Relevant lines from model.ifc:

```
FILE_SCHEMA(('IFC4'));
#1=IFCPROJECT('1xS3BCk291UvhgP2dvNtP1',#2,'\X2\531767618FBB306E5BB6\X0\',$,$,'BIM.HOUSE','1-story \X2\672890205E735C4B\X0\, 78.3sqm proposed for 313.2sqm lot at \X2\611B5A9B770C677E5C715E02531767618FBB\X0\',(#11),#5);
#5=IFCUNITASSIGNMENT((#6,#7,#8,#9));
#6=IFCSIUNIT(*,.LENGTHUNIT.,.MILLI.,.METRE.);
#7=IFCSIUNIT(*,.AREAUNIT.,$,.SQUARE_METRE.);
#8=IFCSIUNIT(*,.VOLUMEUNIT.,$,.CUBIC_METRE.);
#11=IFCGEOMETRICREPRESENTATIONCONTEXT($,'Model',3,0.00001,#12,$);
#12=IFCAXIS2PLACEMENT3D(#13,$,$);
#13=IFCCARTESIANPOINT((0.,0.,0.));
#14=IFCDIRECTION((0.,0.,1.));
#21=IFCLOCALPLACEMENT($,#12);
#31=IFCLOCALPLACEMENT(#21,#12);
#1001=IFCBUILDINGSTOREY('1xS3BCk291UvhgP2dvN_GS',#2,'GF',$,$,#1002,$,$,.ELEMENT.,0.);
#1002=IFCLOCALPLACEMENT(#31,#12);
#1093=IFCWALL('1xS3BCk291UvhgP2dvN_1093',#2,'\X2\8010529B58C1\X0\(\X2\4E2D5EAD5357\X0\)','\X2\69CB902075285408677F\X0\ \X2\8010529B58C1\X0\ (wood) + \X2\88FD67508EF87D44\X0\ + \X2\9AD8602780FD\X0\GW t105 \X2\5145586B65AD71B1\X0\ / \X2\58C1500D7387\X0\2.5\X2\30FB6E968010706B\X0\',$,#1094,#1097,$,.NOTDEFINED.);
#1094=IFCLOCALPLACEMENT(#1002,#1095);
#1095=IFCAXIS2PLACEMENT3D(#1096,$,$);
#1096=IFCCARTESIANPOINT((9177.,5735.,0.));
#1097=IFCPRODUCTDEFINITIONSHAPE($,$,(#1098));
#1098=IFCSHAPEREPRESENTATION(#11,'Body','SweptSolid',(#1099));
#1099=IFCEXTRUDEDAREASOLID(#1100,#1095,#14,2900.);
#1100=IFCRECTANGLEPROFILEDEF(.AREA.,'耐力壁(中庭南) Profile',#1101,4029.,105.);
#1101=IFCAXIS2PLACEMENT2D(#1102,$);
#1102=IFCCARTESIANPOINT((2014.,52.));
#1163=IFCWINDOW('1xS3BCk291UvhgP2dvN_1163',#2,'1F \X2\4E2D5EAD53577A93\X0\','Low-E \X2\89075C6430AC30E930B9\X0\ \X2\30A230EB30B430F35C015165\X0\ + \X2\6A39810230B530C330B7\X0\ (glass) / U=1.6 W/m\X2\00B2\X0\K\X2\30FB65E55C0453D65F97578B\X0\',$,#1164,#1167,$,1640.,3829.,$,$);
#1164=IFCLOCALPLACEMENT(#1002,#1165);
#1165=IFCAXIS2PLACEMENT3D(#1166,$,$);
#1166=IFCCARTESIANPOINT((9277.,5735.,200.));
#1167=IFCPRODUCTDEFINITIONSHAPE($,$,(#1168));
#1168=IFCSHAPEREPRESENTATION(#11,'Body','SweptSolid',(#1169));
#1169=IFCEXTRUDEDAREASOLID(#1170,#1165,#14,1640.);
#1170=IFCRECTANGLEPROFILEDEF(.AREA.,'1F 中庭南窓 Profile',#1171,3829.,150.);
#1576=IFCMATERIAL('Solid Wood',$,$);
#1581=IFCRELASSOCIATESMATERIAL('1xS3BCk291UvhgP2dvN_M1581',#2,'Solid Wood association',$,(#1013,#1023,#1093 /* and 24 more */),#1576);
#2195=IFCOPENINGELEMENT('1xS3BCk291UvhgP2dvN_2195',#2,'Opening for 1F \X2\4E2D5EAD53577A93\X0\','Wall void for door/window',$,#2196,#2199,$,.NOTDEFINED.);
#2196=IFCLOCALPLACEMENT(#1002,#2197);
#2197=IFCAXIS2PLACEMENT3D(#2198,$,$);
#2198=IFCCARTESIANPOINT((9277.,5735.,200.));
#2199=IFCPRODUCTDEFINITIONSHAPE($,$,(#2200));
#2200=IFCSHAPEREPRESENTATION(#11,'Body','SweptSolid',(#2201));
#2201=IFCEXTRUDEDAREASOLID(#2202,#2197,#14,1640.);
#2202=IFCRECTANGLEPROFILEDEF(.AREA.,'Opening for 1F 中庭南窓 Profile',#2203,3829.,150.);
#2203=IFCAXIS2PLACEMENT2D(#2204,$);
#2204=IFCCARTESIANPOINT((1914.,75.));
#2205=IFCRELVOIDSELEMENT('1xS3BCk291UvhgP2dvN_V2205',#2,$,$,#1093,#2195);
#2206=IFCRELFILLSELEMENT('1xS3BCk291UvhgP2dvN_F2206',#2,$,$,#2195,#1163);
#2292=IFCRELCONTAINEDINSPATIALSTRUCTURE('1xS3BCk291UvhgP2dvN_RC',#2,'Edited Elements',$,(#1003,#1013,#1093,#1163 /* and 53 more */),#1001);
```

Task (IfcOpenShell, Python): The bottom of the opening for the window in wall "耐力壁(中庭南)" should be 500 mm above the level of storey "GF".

```python
import numpy as np
import ifcopenshell
import ifcopenshell.api.geometry
import ifcopenshell.geom
import ifcopenshell.util.element
import ifcopenshell.util.placement
import ifcopenshell.util.shape
import ifcopenshell.util.unit

model = ifcopenshell.open("model.ifc")
unit_scale = ifcopenshell.util.unit.calculate_unit_scale(model)

window = model.by_guid("1xS3BCk291UvhgP2dvN_1163")
opening = window.FillsVoids[0].RelatingOpeningElement
storey = ifcopenshell.util.element.get_container(window, ifc_class="IfcBuildingStorey")
level = ifcopenshell.util.placement.get_local_placement(storey.ObjectPlacement)[2, 3]

# The opening's origin need not be at the sill, so measure its lowest point.
shape = ifcopenshell.geom.create_shape(ifcopenshell.geom.settings(), opening)
bottom = ifcopenshell.util.shape.get_shape_bottom_elevation(shape, shape.geometry) / unit_scale
dz = level + 0.5 / unit_scale - bottom

shift = np.array([0.0, 0.0, dz])
# The window is not placed relative to its opening, so move both.
for product in (opening, window):
    matrix = ifcopenshell.util.placement.get_local_placement(product.ObjectPlacement)
    matrix[:3, 3] += shift
    ifcopenshell.api.geometry.edit_object_placement(model, product=product, matrix=matrix, is_si=False)

print(f"moved by {dz * unit_scale:+.3f} m")

model.write("model_v2.ifc")
```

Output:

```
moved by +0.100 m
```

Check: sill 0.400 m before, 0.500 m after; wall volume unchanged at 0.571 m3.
